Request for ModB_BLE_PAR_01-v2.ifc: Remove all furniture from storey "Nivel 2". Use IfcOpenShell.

First a look at what the model holds.

```python
import ifcopenshell
import ifcopenshell.util.element

model = ifcopenshell.open("ModB_BLE_PAR_01-v2.ifc")
print(model.schema)
storey = next(s for s in model.by_type("IfcBuildingStorey") if s.Name == "Nivel 2")
furniture = [e for e in ifcopenshell.util.element.get_decomposition(storey) if e.is_a("IfcFurnishingElement")]
seen = {}
for e in furniture:
    element_type = ifcopenshell.util.element.get_type(e)
    name = element_type.Name if element_type not in (None, e) else None
    seen[name] = seen.get(name, 0) + 1
for name, count in sorted(seen.items(), key=str):
    print(count, "x", name)
```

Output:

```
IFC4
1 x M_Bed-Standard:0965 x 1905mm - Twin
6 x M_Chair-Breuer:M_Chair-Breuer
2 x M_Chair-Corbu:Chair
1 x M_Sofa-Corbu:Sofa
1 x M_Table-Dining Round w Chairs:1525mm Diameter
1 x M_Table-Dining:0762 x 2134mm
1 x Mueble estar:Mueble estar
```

```python
import ifcopenshell
import ifcopenshell.api.root
import ifcopenshell.util.element

model = ifcopenshell.open("ModB_BLE_PAR_01-v2.ifc")

storey = next(s for s in model.by_type("IfcBuildingStorey") if s.Name == "Nivel 2")
furniture = [e for e in ifcopenshell.util.element.get_decomposition(storey) if e.is_a("IfcFurnishingElement")]

for e in furniture:
    ifcopenshell.api.root.remove_product(model, product=e)
print(len(furniture), "removed")

model.write("ModB_BLE_PAR_01-v2_updated.ifc")
```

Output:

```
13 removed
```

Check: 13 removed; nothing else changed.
